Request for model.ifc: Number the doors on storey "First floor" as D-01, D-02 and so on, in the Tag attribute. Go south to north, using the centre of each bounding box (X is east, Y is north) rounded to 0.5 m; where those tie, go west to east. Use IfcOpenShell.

First a look at what the model holds.

```python
import ifcopenshell
import ifcopenshell.util.element
import ifcopenshell.util.placement

model = ifcopenshell.open("model.ifc")
print(model.schema)
storey = next(s for s in model.by_type("IfcBuildingStorey") if s.Name == "First floor")
doors = [e for e in ifcopenshell.util.element.get_decomposition(storey) if e.is_a("IfcDoor")]
for e in sorted(doors, key=lambda e: e.id()):
    origin = ifcopenshell.util.placement.get_local_placement(e.ObjectPlacement)[:3, 3]
    print(e.id(), e.Tag, e.Name, origin.round(2) + 0.0, sep=" | ")
```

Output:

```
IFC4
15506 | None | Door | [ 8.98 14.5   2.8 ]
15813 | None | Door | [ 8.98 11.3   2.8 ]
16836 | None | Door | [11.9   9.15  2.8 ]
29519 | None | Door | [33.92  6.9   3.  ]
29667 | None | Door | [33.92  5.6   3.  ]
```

```python
import ifcopenshell
import ifcopenshell.geom
import ifcopenshell.util.element
import ifcopenshell.util.shape

model = ifcopenshell.open("model.ifc")
settings = ifcopenshell.geom.settings()
settings.set("use-world-coords", True)


def centre(element):
    shape = ifcopenshell.geom.create_shape(settings, element)
    return ifcopenshell.util.shape.get_bbox_centroid(shape.geometry)


storey = next(s for s in model.by_type("IfcBuildingStorey") if s.Name == "First floor")
doors = [e for e in ifcopenshell.util.element.get_decomposition(storey) if e.is_a("IfcDoor")]

# Insertion points can sit at a corner or the storey origin, so sort by the geometry (in metres).
centres = {e: centre(e) for e in doors}
doors.sort(key=lambda e: (round(centres[e][1] / 0.5), centres[e][0]))

for i, e in enumerate(doors, start=1):
    number = f"D-{i:02d}"
    e.Tag = number
    print(e.id(), number)

model.write("model_edited.ifc")
```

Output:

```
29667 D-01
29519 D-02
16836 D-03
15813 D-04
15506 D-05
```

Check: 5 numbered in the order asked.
